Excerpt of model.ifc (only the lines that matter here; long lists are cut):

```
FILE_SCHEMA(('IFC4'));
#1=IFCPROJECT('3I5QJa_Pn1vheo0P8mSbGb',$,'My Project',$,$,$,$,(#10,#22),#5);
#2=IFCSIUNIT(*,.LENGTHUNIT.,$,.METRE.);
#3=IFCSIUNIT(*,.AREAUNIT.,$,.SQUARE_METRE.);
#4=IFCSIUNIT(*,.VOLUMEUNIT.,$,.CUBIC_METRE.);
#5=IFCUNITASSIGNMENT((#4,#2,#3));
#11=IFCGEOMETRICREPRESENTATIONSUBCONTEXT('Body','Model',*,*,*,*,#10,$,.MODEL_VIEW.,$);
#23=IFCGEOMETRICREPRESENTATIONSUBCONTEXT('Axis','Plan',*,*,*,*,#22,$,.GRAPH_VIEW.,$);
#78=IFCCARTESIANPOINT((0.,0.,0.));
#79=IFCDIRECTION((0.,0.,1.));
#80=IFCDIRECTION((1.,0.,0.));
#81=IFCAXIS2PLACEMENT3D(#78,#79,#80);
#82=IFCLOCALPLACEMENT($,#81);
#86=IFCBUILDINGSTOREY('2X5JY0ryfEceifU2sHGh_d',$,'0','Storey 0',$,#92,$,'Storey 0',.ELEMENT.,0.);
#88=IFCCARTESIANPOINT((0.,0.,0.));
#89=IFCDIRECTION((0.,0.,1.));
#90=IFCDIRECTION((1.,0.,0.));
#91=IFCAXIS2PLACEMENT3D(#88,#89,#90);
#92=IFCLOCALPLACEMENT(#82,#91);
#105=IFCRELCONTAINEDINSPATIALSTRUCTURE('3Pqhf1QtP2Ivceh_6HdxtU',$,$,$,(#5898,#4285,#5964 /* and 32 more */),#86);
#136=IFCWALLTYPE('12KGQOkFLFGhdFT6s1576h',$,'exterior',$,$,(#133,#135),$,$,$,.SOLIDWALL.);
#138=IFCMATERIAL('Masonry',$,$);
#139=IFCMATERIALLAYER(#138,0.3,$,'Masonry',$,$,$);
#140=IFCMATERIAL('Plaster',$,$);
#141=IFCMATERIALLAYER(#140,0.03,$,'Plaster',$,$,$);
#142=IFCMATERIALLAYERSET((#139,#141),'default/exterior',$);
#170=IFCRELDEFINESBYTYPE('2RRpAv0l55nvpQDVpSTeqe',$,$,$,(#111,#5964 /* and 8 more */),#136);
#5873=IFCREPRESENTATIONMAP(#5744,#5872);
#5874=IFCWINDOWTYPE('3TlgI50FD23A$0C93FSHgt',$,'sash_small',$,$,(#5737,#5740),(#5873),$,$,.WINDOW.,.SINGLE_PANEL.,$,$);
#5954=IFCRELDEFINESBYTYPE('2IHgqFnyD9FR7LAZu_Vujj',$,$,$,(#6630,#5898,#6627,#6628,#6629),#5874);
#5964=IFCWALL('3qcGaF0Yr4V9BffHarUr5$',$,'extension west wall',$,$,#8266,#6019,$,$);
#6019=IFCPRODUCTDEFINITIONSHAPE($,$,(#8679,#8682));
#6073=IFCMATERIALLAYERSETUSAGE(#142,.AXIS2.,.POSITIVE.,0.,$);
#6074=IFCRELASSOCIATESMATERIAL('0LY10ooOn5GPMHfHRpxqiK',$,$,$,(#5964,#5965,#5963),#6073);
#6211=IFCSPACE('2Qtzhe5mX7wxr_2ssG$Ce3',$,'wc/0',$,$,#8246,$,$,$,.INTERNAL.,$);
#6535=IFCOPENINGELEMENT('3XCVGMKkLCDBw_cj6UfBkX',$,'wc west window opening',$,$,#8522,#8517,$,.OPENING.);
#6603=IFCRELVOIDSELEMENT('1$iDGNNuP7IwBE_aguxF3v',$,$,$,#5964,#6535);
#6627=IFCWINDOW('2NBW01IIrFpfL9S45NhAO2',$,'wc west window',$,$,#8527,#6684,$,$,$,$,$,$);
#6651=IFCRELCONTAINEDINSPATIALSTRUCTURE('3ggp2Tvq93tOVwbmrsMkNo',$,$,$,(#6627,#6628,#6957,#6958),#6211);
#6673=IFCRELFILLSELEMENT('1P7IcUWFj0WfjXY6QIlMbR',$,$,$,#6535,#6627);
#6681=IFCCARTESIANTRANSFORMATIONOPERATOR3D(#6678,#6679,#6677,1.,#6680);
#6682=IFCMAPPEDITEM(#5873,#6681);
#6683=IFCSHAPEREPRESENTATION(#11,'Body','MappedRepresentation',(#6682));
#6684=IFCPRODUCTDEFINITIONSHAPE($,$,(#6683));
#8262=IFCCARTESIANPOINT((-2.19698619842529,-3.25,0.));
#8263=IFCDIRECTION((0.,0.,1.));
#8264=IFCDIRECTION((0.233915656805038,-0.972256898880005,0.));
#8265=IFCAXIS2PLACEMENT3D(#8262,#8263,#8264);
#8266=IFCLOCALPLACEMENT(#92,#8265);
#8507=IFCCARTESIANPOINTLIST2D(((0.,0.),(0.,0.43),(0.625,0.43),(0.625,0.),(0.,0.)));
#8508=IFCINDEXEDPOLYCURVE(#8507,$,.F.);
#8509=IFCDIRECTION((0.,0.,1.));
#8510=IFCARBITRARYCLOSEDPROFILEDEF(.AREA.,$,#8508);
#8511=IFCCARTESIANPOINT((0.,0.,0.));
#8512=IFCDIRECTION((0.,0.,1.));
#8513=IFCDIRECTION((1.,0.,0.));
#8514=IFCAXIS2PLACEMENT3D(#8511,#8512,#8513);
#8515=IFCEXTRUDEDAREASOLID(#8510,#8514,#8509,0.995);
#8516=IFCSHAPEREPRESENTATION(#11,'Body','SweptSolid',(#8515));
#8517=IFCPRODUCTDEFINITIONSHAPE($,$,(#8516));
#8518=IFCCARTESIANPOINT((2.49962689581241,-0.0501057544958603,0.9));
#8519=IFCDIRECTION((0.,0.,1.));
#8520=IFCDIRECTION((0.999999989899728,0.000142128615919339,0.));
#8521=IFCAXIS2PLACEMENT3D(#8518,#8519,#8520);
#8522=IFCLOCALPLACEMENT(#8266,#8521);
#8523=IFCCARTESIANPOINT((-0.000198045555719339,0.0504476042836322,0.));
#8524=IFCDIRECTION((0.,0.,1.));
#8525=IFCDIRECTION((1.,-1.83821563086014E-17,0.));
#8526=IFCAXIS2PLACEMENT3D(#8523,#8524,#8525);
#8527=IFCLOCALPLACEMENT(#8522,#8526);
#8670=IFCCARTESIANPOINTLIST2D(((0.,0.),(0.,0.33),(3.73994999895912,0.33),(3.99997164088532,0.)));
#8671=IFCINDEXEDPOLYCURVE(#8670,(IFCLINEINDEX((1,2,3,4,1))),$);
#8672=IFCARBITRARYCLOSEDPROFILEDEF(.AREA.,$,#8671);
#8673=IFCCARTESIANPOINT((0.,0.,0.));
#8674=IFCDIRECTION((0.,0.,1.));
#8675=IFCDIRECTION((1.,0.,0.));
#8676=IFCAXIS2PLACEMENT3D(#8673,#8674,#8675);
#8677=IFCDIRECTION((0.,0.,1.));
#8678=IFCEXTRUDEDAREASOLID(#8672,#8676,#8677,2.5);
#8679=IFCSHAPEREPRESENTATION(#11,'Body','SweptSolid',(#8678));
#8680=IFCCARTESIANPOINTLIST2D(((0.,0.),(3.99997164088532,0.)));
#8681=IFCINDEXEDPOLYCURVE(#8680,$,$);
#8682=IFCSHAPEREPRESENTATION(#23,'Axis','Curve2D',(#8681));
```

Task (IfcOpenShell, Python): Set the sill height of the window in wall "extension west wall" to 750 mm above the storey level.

```python
import numpy as np
import ifcopenshell
import ifcopenshell.api.geometry
import ifcopenshell.geom
import ifcopenshell.util.element
import ifcopenshell.util.placement
import ifcopenshell.util.shape
import ifcopenshell.util.unit

model = ifcopenshell.open("model.ifc")
unit_scale = ifcopenshell.util.unit.calculate_unit_scale(model)

window = model.by_guid("2NBW01IIrFpfL9S45NhAO2")
opening = window.FillsVoids[0].RelatingOpeningElement
storey = ifcopenshell.util.element.get_container(window, ifc_class="IfcBuildingStorey")
level = ifcopenshell.util.placement.get_local_placement(storey.ObjectPlacement)[2, 3]

# The opening's origin need not be at the sill, so measure its lowest point.
shape = ifcopenshell.geom.create_shape(ifcopenshell.geom.settings(), opening)
bottom = ifcopenshell.util.shape.get_shape_bottom_elevation(shape, shape.geometry) / unit_scale
dz = level + 0.75 - bottom

shift = np.array([0.0, 0.0, dz])
# The window is placed relative to its opening, so it follows when the opening moves.
matrix = ifcopenshell.util.placement.get_local_placement(opening.ObjectPlacement)
matrix[:3, 3] += shift
ifcopenshell.api.geometry.edit_object_placement(
    model, product=opening, matrix=matrix, is_si=False, should_transform_children=True
)

print(f"moved by {dz * unit_scale:+.3f} m")

model.write("model_rev.ifc")
```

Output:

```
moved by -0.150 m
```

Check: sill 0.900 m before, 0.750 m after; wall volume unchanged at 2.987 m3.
